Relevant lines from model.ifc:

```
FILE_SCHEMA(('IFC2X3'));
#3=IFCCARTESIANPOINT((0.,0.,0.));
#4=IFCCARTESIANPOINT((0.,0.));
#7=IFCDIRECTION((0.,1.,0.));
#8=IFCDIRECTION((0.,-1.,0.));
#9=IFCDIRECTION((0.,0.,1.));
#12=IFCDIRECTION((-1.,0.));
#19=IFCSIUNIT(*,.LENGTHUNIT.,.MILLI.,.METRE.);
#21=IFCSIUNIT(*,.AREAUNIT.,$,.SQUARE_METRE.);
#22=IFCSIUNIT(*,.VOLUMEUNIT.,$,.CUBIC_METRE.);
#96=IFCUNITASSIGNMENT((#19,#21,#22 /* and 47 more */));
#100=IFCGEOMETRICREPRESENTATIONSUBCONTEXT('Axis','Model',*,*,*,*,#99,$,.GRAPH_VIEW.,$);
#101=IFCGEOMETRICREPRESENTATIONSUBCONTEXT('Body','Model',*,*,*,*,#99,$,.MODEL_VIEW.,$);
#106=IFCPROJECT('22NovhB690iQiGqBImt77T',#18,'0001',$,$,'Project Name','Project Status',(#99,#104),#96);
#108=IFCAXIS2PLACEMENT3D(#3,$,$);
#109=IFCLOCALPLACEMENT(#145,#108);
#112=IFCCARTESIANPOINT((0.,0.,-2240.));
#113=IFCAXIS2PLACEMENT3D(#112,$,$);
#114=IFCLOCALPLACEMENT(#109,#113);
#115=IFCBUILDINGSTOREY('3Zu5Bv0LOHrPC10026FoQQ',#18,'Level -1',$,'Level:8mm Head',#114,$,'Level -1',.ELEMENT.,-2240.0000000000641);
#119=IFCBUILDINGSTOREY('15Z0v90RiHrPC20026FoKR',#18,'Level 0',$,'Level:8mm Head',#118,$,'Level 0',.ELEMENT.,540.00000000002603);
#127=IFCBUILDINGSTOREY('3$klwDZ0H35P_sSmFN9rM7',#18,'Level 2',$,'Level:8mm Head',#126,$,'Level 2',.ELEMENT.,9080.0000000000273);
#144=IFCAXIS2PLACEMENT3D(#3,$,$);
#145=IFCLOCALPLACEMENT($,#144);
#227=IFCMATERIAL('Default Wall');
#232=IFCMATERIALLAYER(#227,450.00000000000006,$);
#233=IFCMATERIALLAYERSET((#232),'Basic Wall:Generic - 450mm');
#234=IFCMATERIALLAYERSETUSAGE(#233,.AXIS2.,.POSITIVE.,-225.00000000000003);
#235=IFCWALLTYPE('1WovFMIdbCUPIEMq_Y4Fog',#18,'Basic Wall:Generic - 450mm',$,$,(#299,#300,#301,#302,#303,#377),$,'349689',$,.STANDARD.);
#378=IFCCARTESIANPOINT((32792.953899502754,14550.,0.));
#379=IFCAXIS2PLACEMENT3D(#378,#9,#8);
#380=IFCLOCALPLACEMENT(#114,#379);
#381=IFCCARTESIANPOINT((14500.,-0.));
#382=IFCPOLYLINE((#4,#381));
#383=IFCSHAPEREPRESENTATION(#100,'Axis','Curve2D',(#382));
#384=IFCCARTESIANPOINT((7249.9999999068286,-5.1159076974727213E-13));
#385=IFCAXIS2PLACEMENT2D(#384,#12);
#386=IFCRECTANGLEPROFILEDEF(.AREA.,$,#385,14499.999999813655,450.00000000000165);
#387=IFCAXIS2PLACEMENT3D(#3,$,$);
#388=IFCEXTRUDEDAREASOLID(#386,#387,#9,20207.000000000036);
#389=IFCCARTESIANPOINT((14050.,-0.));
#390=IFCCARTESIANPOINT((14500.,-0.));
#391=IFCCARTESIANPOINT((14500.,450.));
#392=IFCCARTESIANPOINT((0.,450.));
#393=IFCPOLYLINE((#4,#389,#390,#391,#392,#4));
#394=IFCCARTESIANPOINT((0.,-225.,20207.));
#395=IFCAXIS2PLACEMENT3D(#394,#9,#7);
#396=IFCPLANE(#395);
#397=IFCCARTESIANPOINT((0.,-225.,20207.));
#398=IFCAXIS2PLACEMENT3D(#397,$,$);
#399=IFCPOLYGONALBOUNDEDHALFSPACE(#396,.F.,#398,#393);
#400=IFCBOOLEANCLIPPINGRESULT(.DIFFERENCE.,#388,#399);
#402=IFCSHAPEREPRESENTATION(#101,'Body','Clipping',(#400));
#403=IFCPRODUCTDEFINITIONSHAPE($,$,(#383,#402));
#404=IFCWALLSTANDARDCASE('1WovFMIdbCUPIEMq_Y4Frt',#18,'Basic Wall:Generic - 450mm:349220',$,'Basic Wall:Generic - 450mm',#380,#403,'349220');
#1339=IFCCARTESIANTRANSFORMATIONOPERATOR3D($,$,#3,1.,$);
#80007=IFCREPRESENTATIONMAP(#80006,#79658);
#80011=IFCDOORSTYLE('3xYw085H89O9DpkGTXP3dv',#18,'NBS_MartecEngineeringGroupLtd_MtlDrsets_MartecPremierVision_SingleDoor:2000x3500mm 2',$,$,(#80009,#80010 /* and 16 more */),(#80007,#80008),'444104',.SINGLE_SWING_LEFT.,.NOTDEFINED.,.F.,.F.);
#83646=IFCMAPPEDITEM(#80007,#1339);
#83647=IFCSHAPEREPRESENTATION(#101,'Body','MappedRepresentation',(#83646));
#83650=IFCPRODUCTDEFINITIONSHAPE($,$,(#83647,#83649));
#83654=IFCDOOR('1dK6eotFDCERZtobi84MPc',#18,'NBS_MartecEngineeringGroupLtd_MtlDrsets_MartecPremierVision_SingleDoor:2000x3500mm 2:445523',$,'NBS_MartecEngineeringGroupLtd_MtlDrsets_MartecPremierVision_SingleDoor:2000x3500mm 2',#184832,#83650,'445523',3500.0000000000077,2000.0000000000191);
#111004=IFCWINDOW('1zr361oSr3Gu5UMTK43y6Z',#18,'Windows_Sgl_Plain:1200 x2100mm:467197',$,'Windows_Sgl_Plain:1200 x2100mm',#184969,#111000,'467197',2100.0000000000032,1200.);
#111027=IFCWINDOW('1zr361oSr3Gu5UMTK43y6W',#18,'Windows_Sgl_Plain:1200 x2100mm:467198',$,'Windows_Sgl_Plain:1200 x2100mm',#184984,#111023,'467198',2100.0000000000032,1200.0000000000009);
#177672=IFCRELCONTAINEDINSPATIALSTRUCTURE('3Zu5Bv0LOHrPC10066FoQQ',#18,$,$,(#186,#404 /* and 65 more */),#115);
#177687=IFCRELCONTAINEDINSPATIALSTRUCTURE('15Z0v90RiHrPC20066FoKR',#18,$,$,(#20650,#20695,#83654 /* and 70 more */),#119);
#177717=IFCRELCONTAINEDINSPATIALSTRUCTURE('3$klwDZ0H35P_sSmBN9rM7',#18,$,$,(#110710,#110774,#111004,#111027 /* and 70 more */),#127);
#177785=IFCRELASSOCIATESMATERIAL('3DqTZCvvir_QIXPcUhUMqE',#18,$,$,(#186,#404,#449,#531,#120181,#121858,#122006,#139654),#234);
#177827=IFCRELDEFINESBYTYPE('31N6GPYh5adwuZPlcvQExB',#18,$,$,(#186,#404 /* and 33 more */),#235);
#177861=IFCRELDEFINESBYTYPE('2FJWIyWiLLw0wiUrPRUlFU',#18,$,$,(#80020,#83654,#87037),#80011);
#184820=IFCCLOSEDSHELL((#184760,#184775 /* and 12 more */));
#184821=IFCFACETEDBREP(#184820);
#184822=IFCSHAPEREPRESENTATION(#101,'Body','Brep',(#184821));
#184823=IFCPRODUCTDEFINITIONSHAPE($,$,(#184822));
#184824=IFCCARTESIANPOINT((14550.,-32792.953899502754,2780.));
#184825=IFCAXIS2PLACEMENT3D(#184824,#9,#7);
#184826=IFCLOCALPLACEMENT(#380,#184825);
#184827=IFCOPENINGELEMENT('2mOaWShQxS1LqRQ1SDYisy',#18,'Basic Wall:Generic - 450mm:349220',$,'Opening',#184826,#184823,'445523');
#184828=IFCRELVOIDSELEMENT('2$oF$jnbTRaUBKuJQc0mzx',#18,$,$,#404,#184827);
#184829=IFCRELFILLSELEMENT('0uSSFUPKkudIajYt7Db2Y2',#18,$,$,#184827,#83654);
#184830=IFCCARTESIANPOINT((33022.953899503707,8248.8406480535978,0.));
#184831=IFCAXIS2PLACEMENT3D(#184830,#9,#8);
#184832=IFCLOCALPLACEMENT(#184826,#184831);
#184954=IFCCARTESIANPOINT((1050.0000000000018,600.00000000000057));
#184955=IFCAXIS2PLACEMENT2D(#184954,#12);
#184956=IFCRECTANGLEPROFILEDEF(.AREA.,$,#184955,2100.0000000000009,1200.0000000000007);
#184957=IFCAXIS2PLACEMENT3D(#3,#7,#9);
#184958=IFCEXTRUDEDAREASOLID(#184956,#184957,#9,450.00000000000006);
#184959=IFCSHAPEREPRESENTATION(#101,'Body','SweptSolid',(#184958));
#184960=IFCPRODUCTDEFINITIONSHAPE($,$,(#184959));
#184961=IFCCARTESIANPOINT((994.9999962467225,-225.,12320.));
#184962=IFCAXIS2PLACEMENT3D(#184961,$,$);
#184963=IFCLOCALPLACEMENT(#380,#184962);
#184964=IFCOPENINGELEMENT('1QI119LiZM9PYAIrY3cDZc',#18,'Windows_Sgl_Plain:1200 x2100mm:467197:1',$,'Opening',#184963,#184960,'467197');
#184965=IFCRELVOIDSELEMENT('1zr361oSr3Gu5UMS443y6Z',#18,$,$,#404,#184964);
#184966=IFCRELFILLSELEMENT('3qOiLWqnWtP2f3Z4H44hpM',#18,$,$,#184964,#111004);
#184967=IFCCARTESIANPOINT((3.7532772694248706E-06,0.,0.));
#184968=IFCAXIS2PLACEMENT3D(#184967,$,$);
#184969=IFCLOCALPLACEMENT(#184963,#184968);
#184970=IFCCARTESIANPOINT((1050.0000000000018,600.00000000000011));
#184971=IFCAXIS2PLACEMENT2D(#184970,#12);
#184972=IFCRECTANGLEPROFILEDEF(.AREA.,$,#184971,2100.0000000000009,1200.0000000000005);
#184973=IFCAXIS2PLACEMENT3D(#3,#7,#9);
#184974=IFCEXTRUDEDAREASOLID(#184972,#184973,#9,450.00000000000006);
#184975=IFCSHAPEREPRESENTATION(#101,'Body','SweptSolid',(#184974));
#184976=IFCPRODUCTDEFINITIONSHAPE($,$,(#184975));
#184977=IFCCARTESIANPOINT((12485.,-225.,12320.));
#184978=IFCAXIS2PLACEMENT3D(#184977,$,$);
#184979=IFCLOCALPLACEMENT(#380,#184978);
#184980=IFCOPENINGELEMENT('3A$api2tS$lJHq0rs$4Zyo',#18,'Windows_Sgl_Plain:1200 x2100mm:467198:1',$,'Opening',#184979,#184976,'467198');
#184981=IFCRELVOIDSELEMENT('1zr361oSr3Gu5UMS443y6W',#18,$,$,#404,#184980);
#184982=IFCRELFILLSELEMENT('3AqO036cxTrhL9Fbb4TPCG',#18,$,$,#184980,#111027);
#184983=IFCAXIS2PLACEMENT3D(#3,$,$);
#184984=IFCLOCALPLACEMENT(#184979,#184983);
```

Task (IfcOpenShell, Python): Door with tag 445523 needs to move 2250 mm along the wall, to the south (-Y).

```python
import ifcopenshell
import ifcopenshell.api.geometry
import ifcopenshell.util.placement
import ifcopenshell.util.unit

model = ifcopenshell.open("model.ifc")
unit_scale = ifcopenshell.util.unit.calculate_unit_scale(model)

door = model.by_guid("1dK6eotFDCERZtobi84MPc")
opening = door.FillsVoids[0].RelatingOpeningElement
wall = opening.VoidsElements[0].RelatingBuildingElement

wall_matrix = ifcopenshell.util.placement.get_local_placement(wall.ObjectPlacement)
shift = wall_matrix[:3, 0] * 2.25 / unit_scale
before = ifcopenshell.util.placement.get_local_placement(door.ObjectPlacement)[:3, 3].copy()

# The door is placed relative to its opening, so it follows when the opening moves.
matrix = ifcopenshell.util.placement.get_local_placement(opening.ObjectPlacement)
matrix[:3, 3] += shift
ifcopenshell.api.geometry.edit_object_placement(
    model, product=opening, matrix=matrix, is_si=False, should_transform_children=True
)

after = ifcopenshell.util.placement.get_local_placement(door.ObjectPlacement)[:3, 3]
print("door moved by", (after - before).round(3) + 0.0)

model.write("model_rev.ifc")
```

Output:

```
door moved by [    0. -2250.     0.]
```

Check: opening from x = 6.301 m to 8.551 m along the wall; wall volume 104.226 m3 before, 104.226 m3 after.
